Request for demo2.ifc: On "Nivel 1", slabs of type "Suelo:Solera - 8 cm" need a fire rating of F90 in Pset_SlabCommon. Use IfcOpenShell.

First a look at what the model holds.

```python
import ifcopenshell
import ifcopenshell.util.element

model = ifcopenshell.open("demo2.ifc")
print(model.schema)
storey = next(s for s in model.by_type("IfcBuildingStorey") if s.Name == "Nivel 1")
slabs = [e for e in ifcopenshell.util.element.get_decomposition(storey) if e.is_a("IfcSlab")]
seen = {}
for e in slabs:
    element_type = ifcopenshell.util.element.get_type(e)
    key = (element_type.Name if element_type != e and element_type else None, ifcopenshell.util.element.get_pset(e, "Pset_SlabCommon", "FireRating"))
    seen[key] = seen.get(key, 0) + 1
for (name, value), count in sorted(seen.items(), key=str):
    print(count, "x", name, "|", value)
```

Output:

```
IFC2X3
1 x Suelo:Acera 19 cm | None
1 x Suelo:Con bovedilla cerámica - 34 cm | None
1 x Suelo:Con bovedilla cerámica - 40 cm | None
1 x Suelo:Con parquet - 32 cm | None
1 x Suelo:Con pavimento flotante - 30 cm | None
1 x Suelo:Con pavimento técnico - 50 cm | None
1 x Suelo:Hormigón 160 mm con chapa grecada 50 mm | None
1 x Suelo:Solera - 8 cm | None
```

```python
import ifcopenshell
import ifcopenshell.api.pset
import ifcopenshell.util.element

model = ifcopenshell.open("demo2.ifc")

storey = next(s for s in model.by_type("IfcBuildingStorey") if s.Name == "Nivel 1")
slabs = [e for e in ifcopenshell.util.element.get_decomposition(storey) if e.is_a("IfcSlab")]

count = 0
for e in slabs:
    element_type = ifcopenshell.util.element.get_type(e)
    if element_type in (None, e) or element_type.Name != "Suelo:Solera - 8 cm":
        continue
    # add_pset returns the element's existing set when there is one.
    pset = ifcopenshell.api.pset.add_pset(model, product=e, name="Pset_SlabCommon")
    ifcopenshell.api.pset.edit_pset(model, pset=pset, properties={"FireRating": "F90"})
    count += 1

print(count, "slabs updated")

model.write("demo2_v2.ifc")
```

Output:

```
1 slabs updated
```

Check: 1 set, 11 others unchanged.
